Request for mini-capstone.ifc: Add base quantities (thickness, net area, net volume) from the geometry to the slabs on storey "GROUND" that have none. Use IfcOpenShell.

First a look at what the model holds.

```python
import ifcopenshell
import ifcopenshell.util.element
import ifcopenshell.util.unit

model = ifcopenshell.open("mini-capstone.ifc")
print(model.schema)
for unit_type in ("LENGTHUNIT", "AREAUNIT", "VOLUMEUNIT"):
    print(unit_type, ifcopenshell.util.unit.calculate_unit_scale(model, unit_type))
storey = next(s for s in model.by_type("IfcBuildingStorey") if s.Name == "GROUND")
slabs = [e for e in ifcopenshell.util.element.get_decomposition(storey) if e.is_a("IfcSlab")]
for e in sorted(slabs, key=lambda e: e.id()):
    print(e.id(), e.is_a(), e.Name, list(ifcopenshell.util.element.get_psets(e, qtos_only=True)), sep=" | ")
```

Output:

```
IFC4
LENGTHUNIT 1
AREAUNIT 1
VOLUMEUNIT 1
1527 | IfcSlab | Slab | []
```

```python
import ifcopenshell
import ifcopenshell.api.pset
import ifcopenshell.geom
import ifcopenshell.util.element
import ifcopenshell.util.shape
import ifcopenshell.util.unit

model = ifcopenshell.open("mini-capstone.ifc")
unit_scale = ifcopenshell.util.unit.calculate_unit_scale(model)
area_scale = ifcopenshell.util.unit.calculate_unit_scale(model, "AREAUNIT")
volume_scale = ifcopenshell.util.unit.calculate_unit_scale(model, "VOLUMEUNIT")
settings = ifcopenshell.geom.settings()

storey = next(s for s in model.by_type("IfcBuildingStorey") if s.Name == "GROUND")
slabs = [e for e in ifcopenshell.util.element.get_decomposition(storey) if e.is_a("IfcSlab")]

for e in sorted(slabs, key=lambda e: e.id()):
    if ifcopenshell.util.element.get_psets(e, qtos_only=True, should_inherit=False):
        continue
    # Geometry comes back in metres, in the element's own axes.
    shape = ifcopenshell.geom.create_shape(settings, e)
    values = {
        "Width": ifcopenshell.util.shape.get_z(shape.geometry) / unit_scale,
        "NetArea": ifcopenshell.util.shape.get_footprint_area(shape.geometry) / area_scale,
        "NetVolume": ifcopenshell.util.shape.get_volume(shape.geometry) / volume_scale,
    }
    qto = ifcopenshell.api.pset.add_qto(model, product=e, name="Qto_SlabBaseQuantities")
    ifcopenshell.api.pset.edit_qto(model, qto=qto, properties=values)
    print(e.id(), {k: round(v, 3) for k, v in values.items()})

model.write("mini-capstone_rev.ifc")
```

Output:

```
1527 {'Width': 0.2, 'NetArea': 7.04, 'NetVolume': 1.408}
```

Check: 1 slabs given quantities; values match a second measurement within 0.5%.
